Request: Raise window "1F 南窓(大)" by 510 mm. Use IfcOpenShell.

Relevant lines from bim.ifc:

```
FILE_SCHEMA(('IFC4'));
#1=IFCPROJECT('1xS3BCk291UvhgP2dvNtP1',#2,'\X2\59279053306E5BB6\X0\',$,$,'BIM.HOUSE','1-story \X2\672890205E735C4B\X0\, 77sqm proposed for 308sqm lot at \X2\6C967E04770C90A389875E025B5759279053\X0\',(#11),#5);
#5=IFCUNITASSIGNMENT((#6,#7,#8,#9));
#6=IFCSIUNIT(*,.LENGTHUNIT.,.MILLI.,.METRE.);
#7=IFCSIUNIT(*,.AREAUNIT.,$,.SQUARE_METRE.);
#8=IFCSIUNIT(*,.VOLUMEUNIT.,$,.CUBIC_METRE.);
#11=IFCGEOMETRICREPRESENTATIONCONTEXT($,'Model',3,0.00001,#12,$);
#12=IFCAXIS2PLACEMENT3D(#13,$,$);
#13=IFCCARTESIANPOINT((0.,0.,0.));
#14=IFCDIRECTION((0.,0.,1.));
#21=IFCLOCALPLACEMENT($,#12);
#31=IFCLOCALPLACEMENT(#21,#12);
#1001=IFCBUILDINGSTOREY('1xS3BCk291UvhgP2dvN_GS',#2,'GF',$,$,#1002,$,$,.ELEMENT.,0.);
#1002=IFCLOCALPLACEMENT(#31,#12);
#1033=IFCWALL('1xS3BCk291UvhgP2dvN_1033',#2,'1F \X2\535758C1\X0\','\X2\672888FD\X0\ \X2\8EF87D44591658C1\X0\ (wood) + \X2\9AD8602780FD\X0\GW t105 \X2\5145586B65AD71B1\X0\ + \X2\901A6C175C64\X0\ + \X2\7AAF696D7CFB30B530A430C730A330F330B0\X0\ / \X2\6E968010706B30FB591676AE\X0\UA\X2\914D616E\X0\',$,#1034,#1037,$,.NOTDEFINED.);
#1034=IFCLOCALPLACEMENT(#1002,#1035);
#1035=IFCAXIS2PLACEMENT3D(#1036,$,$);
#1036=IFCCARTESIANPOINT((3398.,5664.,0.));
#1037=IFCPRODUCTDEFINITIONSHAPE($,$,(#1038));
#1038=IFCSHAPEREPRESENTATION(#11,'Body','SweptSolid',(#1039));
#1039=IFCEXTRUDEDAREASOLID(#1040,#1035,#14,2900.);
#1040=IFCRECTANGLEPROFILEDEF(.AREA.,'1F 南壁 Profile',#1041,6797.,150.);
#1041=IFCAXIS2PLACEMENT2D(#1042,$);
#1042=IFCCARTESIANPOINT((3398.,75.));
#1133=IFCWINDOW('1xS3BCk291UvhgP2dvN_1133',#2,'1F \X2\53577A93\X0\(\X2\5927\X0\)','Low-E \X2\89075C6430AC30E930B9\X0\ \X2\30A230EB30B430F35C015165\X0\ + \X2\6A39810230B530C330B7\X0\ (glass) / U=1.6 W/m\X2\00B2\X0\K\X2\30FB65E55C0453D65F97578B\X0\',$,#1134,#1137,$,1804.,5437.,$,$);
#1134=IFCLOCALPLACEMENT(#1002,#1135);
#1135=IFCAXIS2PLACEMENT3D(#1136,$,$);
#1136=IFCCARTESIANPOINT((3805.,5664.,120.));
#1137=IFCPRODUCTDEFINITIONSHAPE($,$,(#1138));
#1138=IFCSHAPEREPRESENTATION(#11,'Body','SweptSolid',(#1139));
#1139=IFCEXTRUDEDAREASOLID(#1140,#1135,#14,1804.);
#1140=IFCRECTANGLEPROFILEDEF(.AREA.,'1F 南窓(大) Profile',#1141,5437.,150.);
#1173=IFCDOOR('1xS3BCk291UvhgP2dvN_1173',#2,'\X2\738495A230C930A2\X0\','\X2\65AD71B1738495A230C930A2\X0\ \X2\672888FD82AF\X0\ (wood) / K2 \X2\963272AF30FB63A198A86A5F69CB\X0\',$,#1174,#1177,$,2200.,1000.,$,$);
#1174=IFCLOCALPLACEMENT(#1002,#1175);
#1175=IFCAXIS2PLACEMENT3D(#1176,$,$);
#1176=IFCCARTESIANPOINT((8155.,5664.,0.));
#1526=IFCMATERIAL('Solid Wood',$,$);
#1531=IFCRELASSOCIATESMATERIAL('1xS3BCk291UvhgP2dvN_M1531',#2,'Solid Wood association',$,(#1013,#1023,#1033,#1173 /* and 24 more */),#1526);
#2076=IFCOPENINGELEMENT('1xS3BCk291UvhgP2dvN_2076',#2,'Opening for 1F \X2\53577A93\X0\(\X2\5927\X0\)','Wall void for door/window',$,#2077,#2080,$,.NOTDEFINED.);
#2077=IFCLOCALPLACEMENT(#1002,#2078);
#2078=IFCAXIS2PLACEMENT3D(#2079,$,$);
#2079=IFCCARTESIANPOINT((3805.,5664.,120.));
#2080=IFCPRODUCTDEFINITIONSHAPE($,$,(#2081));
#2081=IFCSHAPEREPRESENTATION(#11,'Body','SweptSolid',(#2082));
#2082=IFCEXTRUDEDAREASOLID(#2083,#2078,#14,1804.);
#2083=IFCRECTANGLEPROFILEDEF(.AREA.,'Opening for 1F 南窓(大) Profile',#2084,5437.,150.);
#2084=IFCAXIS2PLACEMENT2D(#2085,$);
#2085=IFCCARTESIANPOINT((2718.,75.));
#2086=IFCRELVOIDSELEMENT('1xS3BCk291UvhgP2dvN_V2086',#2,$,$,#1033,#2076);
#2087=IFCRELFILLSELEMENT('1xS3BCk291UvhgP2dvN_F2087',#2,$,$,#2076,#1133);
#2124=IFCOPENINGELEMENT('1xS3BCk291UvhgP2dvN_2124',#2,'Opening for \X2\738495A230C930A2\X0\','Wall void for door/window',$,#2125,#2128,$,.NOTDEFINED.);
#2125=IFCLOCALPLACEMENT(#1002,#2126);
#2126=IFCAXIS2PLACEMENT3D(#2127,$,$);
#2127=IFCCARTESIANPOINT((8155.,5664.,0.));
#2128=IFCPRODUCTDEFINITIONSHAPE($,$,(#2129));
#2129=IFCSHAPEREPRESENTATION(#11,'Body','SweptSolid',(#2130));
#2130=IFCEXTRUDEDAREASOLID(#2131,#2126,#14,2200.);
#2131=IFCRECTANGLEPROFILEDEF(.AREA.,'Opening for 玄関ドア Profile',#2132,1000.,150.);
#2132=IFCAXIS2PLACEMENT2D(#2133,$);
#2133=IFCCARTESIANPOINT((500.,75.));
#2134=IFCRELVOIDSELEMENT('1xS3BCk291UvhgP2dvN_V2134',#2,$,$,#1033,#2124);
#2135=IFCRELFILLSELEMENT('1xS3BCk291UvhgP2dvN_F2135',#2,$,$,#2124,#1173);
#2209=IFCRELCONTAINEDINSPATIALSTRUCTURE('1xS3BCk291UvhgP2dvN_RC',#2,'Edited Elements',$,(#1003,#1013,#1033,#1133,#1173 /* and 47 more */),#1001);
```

```python
import numpy as np
import ifcopenshell
import ifcopenshell.api.geometry
import ifcopenshell.util.placement
import ifcopenshell.util.unit

model = ifcopenshell.open("bim.ifc")
unit_scale = ifcopenshell.util.unit.calculate_unit_scale(model)

window = model.by_id(1133)
opening = window.FillsVoids[0].RelatingOpeningElement
dz = 510.0

shift = np.array([0.0, 0.0, dz])
# The window is not placed relative to its opening, so move both.
for product in (opening, window):
    matrix = ifcopenshell.util.placement.get_local_placement(product.ObjectPlacement)
    matrix[:3, 3] += shift
    ifcopenshell.api.geometry.edit_object_placement(model, product=product, matrix=matrix, is_si=False)

print(f"moved by {dz * unit_scale:+.3f} m")

model.write("bim_v2.ifc")
```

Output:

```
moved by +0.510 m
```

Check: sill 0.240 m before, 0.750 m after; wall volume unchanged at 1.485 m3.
